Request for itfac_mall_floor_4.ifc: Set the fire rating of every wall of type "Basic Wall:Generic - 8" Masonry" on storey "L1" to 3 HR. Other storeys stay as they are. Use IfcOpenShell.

First a look at what the model holds.

```python
import ifcopenshell
import ifcopenshell.util.element

model = ifcopenshell.open("itfac_mall_floor_4.ifc")
print(model.schema)
storey = next(s for s in model.by_type("IfcBuildingStorey") if s.Name == "L1")
walls = [e for e in ifcopenshell.util.element.get_decomposition(storey) if e.is_a("IfcWall")]
seen = {}
for e in walls:
    element_type = ifcopenshell.util.element.get_type(e)
    key = (element_type.Name if element_type != e and element_type else None, ifcopenshell.util.element.get_pset(e, "Pset_WallCommon", "FireRating"))
    seen[key] = seen.get(key, 0) + 1
for (name, value), count in sorted(seen.items(), key=str):
    print(count, "x", name, "|", value)
```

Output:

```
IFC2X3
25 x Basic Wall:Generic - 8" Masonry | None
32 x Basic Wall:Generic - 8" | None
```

```python
import ifcopenshell
import ifcopenshell.api.pset
import ifcopenshell.util.element

model = ifcopenshell.open("itfac_mall_floor_4.ifc")

storey = next(s for s in model.by_type("IfcBuildingStorey") if s.Name == "L1")
walls = [e for e in ifcopenshell.util.element.get_decomposition(storey) if e.is_a("IfcWall")]

count = 0
for e in walls:
    element_type = ifcopenshell.util.element.get_type(e)
    if element_type in (None, e) or element_type.Name != 'Basic Wall:Generic - 8" Masonry':
        continue
    # add_pset returns the element's existing set when there is one.
    pset = ifcopenshell.api.pset.add_pset(model, product=e, name="Pset_WallCommon")
    ifcopenshell.api.pset.edit_pset(model, pset=pset, properties={"FireRating": "3 HR"})
    count += 1

print(count, "walls updated")

model.write("itfac_mall_floor_4_edited.ifc")
```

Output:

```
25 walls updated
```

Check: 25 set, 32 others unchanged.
